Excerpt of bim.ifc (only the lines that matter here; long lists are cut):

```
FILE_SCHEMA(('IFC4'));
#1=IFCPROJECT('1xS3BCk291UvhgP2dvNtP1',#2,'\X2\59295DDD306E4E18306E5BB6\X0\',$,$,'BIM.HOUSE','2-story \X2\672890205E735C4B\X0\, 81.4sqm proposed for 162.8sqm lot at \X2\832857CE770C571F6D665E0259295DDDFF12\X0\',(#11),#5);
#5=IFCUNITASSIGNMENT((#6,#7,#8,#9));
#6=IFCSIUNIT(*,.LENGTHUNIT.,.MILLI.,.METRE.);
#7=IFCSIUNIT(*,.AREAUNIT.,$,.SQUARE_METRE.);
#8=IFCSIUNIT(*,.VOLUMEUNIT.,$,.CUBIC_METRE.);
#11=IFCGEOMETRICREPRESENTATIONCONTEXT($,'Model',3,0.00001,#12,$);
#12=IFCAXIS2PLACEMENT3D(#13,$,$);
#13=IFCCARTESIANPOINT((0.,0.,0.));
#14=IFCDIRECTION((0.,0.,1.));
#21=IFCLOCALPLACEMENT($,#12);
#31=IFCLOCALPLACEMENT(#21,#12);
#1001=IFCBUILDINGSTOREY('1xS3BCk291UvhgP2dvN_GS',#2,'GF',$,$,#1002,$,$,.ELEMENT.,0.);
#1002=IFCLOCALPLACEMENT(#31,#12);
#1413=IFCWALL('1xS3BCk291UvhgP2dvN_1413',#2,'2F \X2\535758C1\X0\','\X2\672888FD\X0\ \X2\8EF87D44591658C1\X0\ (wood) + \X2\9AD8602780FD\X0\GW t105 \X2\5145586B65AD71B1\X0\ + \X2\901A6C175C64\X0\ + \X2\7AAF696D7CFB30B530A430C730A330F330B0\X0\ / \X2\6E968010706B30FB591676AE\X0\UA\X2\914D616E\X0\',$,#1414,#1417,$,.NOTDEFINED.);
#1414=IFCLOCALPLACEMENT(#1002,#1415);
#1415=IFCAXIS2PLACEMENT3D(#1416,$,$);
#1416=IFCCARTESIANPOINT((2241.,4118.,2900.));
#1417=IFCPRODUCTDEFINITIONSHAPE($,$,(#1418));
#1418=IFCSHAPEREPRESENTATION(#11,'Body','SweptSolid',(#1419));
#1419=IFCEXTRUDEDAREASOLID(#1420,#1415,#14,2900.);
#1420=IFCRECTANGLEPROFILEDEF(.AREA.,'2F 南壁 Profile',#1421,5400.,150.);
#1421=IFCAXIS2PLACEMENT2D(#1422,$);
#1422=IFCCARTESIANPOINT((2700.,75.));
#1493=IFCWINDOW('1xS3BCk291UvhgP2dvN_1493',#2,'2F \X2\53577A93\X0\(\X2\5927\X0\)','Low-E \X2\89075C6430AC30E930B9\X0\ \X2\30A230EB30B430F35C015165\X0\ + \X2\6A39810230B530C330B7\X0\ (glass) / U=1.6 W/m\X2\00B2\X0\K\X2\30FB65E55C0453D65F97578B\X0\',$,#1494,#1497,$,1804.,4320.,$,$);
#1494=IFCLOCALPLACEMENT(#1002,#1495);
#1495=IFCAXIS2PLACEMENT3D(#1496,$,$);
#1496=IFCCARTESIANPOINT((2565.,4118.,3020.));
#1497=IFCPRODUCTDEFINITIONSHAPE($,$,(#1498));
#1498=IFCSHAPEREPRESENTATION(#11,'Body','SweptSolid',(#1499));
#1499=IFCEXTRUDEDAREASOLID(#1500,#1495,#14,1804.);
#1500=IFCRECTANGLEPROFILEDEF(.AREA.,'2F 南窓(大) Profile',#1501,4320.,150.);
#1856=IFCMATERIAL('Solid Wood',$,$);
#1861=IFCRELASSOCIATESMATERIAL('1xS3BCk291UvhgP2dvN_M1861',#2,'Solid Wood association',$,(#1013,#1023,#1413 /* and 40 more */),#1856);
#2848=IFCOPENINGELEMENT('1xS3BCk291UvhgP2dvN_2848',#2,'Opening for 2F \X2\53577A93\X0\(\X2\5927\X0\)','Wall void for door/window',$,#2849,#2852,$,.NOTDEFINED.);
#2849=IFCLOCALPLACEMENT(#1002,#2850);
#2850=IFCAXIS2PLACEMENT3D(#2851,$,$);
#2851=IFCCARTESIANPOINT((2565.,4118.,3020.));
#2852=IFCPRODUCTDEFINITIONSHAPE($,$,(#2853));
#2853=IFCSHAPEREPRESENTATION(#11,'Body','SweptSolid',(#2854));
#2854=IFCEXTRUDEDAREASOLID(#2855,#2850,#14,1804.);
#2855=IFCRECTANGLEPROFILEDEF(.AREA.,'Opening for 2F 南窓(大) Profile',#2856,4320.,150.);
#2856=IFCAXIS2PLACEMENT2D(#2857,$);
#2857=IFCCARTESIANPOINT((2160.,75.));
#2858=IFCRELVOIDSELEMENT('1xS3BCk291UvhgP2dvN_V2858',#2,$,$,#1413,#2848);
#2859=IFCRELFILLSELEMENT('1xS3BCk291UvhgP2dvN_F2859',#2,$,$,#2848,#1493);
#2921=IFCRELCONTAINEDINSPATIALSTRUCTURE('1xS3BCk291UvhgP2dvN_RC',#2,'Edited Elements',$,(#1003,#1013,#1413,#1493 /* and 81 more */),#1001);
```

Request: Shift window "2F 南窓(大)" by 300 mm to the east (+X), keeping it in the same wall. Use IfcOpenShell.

```python
import ifcopenshell
import ifcopenshell.api.geometry
import ifcopenshell.util.placement
import ifcopenshell.util.unit

model = ifcopenshell.open("bim.ifc")
unit_scale = ifcopenshell.util.unit.calculate_unit_scale(model)

window = model.by_guid("1xS3BCk291UvhgP2dvN_1493")
opening = window.FillsVoids[0].RelatingOpeningElement
wall = opening.VoidsElements[0].RelatingBuildingElement

wall_matrix = ifcopenshell.util.placement.get_local_placement(wall.ObjectPlacement)
shift = wall_matrix[:3, 0] * 0.3 / unit_scale
before = ifcopenshell.util.placement.get_local_placement(window.ObjectPlacement)[:3, 3].copy()

# The window is not placed relative to its opening, so move both.
for product in (opening, window):
    matrix = ifcopenshell.util.placement.get_local_placement(product.ObjectPlacement)
    matrix[:3, 3] += shift
    ifcopenshell.api.geometry.edit_object_placement(model, product=product, matrix=matrix, is_si=False)

after = ifcopenshell.util.placement.get_local_placement(window.ObjectPlacement)[:3, 3]
print("window moved by", (after - before).round(3) + 0.0)

model.write("bim_v2.ifc")
```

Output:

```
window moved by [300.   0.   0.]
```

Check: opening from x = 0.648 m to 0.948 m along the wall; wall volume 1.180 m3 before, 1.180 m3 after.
